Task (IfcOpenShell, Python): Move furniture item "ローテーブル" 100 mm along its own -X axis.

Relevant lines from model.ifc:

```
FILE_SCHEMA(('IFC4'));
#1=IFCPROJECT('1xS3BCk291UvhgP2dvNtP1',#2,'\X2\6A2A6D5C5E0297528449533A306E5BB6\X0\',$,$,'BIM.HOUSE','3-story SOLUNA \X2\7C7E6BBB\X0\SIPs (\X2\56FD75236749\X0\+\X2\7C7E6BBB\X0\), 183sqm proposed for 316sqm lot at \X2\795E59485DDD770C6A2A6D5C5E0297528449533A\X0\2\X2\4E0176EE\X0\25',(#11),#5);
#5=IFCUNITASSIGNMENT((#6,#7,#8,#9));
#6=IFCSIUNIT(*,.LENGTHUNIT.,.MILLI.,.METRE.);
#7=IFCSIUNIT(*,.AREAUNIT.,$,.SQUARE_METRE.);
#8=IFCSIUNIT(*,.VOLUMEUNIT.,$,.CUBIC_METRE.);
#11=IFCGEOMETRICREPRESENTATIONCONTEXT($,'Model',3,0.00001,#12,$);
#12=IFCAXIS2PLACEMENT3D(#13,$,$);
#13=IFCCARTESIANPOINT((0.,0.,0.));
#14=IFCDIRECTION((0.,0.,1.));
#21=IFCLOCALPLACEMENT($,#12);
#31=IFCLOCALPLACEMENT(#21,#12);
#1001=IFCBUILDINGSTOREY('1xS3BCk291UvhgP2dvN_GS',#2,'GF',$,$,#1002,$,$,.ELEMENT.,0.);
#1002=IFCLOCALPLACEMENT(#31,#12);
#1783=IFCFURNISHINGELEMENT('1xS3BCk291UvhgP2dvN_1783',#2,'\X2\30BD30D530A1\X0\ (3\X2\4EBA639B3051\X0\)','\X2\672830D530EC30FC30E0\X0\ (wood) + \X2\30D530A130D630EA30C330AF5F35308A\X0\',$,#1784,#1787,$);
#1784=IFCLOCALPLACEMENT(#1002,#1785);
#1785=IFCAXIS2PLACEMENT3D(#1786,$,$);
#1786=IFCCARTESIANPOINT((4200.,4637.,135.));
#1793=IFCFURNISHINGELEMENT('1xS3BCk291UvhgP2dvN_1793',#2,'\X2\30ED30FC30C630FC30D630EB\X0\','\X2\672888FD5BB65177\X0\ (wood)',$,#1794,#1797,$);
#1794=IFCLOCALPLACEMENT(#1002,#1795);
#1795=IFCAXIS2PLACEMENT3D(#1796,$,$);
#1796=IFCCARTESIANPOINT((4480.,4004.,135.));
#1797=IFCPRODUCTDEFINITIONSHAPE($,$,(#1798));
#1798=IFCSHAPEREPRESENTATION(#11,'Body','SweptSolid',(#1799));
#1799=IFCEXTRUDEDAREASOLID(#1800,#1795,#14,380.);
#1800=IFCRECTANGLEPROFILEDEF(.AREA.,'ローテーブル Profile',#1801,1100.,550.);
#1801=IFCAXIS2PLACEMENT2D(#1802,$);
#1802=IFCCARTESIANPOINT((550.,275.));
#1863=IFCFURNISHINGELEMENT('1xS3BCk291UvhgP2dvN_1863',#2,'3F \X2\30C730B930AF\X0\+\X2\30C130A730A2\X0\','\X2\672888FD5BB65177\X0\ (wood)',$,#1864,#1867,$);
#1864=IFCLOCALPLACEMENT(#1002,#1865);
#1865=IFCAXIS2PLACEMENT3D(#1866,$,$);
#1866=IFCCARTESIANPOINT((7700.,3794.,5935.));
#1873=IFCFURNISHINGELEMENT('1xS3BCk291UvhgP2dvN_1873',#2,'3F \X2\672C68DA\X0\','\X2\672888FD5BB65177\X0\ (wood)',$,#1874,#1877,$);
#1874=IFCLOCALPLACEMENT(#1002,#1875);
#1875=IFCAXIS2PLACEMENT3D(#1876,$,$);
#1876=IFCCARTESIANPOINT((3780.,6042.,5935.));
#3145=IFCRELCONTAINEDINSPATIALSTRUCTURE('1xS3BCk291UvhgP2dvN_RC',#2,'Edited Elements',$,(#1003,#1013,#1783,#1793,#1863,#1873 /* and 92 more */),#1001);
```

```python
import ifcopenshell
import ifcopenshell.api.geometry
import ifcopenshell.util.placement

model = ifcopenshell.open("model.ifc")

item = model.by_guid("1xS3BCk291UvhgP2dvN_1793")
matrix = ifcopenshell.util.placement.get_local_placement(item.ObjectPlacement)
matrix[:3, 3] -= matrix[:3, 0] * 100.0
ifcopenshell.api.geometry.edit_object_placement(model, product=item, matrix=matrix, is_si=False)

print(ifcopenshell.util.placement.get_local_placement(item.ObjectPlacement).round(3) + 0.0)

model.write("model_updated.ifc")
```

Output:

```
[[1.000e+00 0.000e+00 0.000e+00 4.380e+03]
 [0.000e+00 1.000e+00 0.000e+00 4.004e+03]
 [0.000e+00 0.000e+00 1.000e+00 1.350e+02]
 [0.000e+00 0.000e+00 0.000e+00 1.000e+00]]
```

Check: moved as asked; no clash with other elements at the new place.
